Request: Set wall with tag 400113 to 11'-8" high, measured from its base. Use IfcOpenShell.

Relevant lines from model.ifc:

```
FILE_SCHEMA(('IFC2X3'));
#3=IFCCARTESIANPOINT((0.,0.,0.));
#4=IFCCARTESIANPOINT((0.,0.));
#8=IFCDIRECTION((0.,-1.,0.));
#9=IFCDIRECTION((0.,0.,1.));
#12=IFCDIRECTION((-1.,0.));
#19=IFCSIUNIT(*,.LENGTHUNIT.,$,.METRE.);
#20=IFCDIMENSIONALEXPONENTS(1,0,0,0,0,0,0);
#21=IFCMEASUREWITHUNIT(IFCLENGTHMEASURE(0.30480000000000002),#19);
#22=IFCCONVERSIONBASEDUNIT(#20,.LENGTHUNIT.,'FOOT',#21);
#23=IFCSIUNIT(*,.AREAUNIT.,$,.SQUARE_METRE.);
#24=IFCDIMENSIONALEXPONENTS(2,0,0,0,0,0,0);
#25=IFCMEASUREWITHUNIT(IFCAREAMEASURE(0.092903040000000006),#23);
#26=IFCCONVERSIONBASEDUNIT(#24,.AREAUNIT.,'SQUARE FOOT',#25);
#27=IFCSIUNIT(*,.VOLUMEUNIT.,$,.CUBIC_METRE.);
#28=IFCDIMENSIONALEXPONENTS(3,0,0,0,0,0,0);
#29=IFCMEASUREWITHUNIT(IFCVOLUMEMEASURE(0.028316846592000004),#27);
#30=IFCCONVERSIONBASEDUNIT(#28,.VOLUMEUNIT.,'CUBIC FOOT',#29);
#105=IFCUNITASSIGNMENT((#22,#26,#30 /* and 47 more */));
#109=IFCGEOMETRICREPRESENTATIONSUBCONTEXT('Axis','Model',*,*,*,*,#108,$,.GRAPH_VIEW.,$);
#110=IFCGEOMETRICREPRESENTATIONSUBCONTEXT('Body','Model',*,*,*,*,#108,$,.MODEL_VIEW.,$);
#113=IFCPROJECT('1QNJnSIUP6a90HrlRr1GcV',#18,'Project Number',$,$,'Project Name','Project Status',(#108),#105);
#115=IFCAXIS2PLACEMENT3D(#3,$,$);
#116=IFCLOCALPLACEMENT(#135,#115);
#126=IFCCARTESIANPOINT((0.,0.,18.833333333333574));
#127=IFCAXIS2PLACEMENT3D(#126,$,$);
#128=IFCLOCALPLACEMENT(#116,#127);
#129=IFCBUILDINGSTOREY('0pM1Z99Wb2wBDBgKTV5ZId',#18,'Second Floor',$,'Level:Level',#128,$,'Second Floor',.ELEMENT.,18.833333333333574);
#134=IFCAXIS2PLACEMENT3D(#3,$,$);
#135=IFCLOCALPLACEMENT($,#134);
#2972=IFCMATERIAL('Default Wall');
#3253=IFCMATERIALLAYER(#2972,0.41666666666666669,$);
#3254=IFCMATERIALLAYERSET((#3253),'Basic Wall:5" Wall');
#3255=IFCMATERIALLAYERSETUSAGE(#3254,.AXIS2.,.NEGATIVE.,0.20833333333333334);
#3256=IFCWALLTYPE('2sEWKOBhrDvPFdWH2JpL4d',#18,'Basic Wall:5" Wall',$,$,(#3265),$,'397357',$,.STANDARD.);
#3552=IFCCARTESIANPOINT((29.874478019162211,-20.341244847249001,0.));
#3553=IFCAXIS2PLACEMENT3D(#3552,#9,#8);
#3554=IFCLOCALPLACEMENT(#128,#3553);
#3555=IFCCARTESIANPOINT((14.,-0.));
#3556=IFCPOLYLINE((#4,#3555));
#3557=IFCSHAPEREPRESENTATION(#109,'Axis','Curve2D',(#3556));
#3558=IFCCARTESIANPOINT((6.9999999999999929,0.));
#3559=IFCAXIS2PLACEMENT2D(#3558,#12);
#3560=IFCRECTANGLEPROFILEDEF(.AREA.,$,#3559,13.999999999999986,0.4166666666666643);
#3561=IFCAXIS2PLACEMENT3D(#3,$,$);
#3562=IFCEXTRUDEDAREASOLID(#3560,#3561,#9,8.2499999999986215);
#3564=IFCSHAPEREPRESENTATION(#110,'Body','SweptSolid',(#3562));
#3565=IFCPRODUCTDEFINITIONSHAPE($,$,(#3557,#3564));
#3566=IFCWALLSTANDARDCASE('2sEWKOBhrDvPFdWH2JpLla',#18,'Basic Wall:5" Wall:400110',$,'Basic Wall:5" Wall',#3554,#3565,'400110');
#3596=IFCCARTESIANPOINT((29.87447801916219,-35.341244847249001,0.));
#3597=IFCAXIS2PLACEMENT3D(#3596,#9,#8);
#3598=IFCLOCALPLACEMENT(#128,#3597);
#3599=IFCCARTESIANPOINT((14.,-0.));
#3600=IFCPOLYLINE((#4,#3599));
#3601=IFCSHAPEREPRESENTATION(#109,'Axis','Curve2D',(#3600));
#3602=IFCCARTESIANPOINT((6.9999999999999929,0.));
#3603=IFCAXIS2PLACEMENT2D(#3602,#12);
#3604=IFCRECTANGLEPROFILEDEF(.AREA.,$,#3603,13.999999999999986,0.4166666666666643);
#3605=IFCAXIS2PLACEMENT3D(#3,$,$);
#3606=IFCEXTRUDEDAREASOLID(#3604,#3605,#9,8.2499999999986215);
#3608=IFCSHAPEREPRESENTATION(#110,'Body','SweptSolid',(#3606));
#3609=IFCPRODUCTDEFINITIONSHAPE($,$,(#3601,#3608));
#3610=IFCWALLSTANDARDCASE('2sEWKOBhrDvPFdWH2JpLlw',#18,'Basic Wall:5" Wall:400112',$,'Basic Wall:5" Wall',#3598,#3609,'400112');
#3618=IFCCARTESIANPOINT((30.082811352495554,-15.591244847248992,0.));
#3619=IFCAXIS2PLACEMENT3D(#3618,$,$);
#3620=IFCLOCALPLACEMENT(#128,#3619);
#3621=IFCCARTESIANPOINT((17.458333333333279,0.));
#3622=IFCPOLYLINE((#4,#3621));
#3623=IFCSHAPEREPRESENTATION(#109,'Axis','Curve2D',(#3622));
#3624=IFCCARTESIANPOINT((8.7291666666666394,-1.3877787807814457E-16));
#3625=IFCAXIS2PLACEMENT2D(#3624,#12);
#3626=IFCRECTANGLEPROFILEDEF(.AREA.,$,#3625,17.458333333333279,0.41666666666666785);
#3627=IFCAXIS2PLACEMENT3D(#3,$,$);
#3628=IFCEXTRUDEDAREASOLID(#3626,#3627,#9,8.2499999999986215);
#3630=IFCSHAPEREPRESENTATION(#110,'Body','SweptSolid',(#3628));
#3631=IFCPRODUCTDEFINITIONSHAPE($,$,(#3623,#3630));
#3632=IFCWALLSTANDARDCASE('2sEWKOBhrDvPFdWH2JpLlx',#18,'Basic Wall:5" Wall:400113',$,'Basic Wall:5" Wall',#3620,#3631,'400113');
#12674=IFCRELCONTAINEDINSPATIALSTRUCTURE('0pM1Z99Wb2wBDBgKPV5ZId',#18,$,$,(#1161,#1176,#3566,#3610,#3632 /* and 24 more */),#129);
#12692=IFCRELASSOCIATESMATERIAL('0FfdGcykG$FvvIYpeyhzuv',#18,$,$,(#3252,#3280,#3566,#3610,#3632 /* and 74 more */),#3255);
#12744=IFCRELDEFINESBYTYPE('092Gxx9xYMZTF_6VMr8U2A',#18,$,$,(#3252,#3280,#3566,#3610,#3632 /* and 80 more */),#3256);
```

```python
import ifcopenshell
import ifcopenshell.geom
import ifcopenshell.util.representation
import ifcopenshell.util.shape
import ifcopenshell.util.unit

model = ifcopenshell.open("model.ifc")
unit_scale = ifcopenshell.util.unit.calculate_unit_scale(model)
settings = ifcopenshell.geom.settings()


def volume(element):
    """Net volume in cubic metres, openings subtracted."""
    shape = ifcopenshell.geom.create_shape(settings, element)
    return ifcopenshell.util.shape.get_volume(shape.geometry)


wall = model.by_id(3632)
before = volume(wall)

body = ifcopenshell.util.representation.get_representation(wall, "Model", "Body")
solid = body.Items[0]
old_height = solid.Depth
solid.Depth = 140 * 0.0254 / unit_scale
after = volume(wall)

print(f"height {old_height:g} -> {solid.Depth:g}, volume {before:.3f} -> {after:.3f} m3")

model.write("model_updated.ifc")
```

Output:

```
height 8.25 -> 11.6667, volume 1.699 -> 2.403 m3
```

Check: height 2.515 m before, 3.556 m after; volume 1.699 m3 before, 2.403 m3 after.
